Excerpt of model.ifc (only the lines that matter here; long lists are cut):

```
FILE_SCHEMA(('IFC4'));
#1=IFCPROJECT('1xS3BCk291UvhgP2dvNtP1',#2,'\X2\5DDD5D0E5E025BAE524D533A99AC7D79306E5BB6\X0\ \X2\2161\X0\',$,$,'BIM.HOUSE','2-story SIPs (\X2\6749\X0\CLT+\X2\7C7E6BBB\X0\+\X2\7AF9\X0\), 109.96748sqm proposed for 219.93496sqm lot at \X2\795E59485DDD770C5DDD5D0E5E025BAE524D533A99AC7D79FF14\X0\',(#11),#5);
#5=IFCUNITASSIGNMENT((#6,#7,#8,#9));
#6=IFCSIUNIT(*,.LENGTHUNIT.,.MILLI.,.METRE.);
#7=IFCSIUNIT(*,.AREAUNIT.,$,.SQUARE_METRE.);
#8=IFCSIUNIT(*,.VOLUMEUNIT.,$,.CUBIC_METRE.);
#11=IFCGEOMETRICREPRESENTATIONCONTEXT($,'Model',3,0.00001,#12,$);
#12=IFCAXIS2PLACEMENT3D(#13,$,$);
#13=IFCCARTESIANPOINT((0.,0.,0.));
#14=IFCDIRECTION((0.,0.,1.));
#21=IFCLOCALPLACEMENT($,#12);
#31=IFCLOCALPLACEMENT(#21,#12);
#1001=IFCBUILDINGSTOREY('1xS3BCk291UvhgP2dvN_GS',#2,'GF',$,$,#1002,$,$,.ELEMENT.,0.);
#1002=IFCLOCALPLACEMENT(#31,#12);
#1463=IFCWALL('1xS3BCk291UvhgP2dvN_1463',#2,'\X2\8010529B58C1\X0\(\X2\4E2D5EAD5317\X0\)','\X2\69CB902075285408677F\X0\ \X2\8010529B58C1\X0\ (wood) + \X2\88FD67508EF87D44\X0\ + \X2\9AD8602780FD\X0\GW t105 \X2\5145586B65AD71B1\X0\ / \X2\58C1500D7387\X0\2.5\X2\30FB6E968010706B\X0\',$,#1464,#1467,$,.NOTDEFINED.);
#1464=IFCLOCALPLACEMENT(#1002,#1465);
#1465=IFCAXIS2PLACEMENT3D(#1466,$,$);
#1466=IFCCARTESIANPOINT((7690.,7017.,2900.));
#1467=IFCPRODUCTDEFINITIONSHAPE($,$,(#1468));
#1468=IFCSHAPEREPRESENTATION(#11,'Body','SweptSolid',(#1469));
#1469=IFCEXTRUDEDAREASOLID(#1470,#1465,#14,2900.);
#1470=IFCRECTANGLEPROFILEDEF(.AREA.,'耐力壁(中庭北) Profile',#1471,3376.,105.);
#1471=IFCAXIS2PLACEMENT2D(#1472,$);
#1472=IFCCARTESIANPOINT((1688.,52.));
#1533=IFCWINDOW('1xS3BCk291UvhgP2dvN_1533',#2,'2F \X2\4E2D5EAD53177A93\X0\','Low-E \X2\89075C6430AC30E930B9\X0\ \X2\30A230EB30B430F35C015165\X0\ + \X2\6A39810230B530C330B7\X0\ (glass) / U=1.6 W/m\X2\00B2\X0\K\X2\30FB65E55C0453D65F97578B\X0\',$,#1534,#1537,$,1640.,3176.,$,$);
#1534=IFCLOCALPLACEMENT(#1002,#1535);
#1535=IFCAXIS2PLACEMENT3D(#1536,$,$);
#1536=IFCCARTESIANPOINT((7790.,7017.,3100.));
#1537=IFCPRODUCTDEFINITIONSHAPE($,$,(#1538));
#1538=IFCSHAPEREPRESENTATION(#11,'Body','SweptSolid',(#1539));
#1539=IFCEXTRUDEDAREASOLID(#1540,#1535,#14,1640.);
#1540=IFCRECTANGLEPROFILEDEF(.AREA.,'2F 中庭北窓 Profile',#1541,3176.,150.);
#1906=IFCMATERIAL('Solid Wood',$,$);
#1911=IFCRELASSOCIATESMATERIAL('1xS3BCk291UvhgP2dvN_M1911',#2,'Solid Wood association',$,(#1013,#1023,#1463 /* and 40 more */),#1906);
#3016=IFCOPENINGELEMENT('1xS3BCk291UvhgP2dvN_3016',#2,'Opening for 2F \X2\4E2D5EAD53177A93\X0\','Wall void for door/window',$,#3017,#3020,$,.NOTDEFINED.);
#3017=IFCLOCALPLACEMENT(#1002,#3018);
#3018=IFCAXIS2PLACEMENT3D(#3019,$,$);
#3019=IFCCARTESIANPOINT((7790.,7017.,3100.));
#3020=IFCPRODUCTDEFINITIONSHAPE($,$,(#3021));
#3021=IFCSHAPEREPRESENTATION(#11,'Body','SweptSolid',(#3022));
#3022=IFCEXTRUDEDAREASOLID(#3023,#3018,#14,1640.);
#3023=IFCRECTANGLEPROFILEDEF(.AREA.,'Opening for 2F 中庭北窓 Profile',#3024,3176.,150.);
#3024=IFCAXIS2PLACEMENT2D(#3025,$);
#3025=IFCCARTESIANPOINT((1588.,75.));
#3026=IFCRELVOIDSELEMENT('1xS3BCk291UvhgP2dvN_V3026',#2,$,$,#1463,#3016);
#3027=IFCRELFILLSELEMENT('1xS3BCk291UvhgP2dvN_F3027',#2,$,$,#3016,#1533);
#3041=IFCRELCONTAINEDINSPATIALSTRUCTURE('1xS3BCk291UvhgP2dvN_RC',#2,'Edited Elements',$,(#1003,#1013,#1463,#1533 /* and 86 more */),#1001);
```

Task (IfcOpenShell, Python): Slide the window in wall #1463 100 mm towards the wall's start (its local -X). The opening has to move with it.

```python
import ifcopenshell
import ifcopenshell.api.geometry
import ifcopenshell.util.placement
import ifcopenshell.util.unit

model = ifcopenshell.open("model.ifc")
unit_scale = ifcopenshell.util.unit.calculate_unit_scale(model)

window = model.by_guid("1xS3BCk291UvhgP2dvN_1533")
opening = window.FillsVoids[0].RelatingOpeningElement
wall = opening.VoidsElements[0].RelatingBuildingElement

wall_matrix = ifcopenshell.util.placement.get_local_placement(wall.ObjectPlacement)
shift = wall_matrix[:3, 0] * -0.1 / unit_scale
before = ifcopenshell.util.placement.get_local_placement(window.ObjectPlacement)[:3, 3].copy()

# The window is not placed relative to its opening, so move both.
for product in (opening, window):
    matrix = ifcopenshell.util.placement.get_local_placement(product.ObjectPlacement)
    matrix[:3, 3] += shift
    ifcopenshell.api.geometry.edit_object_placement(model, product=product, matrix=matrix, is_si=False)

after = ifcopenshell.util.placement.get_local_placement(window.ObjectPlacement)[:3, 3]
print("window moved by", (after - before).round(3) + 0.0)

model.write("model_rev.ifc")
```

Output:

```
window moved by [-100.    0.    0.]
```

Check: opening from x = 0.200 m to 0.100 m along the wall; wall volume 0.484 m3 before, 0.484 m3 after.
